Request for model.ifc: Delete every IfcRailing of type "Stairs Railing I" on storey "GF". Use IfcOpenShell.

First a look at what the model holds.

```python
import ifcopenshell
import ifcopenshell.util.element

model = ifcopenshell.open("model.ifc")
print(model.schema)
storey = next(s for s in model.by_type("IfcBuildingStorey") if s.Name == "GF")
railings = [e for e in ifcopenshell.util.element.get_decomposition(storey) if e.is_a("IfcRailing")]
seen = {}
for e in railings:
    element_type = ifcopenshell.util.element.get_type(e)
    name = element_type.Name if element_type not in (None, e) else None
    seen[name] = seen.get(name, 0) + 1
for name, count in sorted(seen.items(), key=str):
    print(count, "x", name)
```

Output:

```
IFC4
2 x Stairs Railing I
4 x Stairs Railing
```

```python
import ifcopenshell
import ifcopenshell.api.root
import ifcopenshell.util.element

model = ifcopenshell.open("model.ifc")

storey = next(s for s in model.by_type("IfcBuildingStorey") if s.Name == "GF")
railings = [e for e in ifcopenshell.util.element.get_decomposition(storey) if e.is_a("IfcRailing")]
targets = [e for e in railings if (t := ifcopenshell.util.element.get_type(e)) not in (None, e) and t.Name == "Stairs Railing I"]

for e in targets:
    ifcopenshell.api.root.remove_product(model, product=e)
print(len(targets), "removed")

model.write("model_v2.ifc")
```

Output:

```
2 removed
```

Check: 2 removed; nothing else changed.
